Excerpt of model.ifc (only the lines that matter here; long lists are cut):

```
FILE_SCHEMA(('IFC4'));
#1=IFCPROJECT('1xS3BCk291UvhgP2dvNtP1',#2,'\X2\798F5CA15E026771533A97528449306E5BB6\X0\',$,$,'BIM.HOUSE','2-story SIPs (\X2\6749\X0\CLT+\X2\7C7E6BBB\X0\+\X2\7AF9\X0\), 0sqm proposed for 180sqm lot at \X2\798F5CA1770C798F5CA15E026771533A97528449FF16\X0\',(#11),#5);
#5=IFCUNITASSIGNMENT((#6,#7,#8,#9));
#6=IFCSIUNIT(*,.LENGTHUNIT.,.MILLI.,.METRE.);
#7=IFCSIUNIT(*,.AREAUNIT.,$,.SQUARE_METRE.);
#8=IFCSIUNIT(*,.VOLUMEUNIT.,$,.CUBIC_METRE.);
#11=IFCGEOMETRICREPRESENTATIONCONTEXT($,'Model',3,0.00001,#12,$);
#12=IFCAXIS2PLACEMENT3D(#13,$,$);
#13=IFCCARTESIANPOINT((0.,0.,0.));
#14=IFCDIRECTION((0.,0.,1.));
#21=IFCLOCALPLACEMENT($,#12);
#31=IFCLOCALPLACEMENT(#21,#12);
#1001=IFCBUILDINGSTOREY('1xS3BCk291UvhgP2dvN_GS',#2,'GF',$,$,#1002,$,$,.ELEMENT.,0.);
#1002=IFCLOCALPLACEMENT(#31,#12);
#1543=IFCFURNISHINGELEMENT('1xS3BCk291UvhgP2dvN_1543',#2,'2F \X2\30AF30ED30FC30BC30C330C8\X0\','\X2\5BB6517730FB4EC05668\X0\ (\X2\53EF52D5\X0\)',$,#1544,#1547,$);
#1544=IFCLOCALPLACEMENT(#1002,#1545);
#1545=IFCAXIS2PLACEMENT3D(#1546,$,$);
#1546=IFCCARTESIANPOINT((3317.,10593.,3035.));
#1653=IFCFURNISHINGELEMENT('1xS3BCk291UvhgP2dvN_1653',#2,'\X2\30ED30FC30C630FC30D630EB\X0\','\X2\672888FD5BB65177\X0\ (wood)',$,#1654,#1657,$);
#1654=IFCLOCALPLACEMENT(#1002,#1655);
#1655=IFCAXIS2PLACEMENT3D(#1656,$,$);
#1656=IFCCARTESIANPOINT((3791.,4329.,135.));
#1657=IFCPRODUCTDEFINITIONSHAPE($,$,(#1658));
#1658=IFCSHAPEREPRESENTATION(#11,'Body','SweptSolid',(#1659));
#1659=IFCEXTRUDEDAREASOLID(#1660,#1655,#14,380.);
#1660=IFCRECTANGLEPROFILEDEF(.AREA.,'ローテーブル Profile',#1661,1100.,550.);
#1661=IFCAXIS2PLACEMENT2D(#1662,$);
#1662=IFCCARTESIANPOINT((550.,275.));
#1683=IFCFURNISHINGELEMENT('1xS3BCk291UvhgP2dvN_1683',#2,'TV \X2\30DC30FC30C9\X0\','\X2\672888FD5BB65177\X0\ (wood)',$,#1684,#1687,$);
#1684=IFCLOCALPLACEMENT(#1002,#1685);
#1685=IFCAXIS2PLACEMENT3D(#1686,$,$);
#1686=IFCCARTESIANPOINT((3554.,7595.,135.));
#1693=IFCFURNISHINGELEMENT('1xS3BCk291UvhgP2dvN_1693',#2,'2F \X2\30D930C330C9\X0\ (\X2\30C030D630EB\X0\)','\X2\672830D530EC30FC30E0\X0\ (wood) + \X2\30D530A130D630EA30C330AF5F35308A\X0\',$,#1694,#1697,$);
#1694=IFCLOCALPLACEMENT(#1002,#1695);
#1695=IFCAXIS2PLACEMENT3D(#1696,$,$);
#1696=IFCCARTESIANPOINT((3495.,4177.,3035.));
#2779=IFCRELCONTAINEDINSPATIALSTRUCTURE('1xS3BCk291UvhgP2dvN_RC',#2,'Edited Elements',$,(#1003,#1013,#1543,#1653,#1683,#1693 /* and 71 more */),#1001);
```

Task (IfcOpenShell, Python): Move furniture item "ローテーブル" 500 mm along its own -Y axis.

```python
import ifcopenshell
import ifcopenshell.api.geometry
import ifcopenshell.util.placement
import ifcopenshell.util.unit

model = ifcopenshell.open("model.ifc")
unit_scale = ifcopenshell.util.unit.calculate_unit_scale(model)

item = model.by_guid("1xS3BCk291UvhgP2dvN_1653")
matrix = ifcopenshell.util.placement.get_local_placement(item.ObjectPlacement)
matrix[:3, 3] -= matrix[:3, 1] * 0.5 / unit_scale
ifcopenshell.api.geometry.edit_object_placement(model, product=item, matrix=matrix, is_si=False)

print(ifcopenshell.util.placement.get_local_placement(item.ObjectPlacement).round(3) + 0.0)

model.write("model_updated.ifc")
```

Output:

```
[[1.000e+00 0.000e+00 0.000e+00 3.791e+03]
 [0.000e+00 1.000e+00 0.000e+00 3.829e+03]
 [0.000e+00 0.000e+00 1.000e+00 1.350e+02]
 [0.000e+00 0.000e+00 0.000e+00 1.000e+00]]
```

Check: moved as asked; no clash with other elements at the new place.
